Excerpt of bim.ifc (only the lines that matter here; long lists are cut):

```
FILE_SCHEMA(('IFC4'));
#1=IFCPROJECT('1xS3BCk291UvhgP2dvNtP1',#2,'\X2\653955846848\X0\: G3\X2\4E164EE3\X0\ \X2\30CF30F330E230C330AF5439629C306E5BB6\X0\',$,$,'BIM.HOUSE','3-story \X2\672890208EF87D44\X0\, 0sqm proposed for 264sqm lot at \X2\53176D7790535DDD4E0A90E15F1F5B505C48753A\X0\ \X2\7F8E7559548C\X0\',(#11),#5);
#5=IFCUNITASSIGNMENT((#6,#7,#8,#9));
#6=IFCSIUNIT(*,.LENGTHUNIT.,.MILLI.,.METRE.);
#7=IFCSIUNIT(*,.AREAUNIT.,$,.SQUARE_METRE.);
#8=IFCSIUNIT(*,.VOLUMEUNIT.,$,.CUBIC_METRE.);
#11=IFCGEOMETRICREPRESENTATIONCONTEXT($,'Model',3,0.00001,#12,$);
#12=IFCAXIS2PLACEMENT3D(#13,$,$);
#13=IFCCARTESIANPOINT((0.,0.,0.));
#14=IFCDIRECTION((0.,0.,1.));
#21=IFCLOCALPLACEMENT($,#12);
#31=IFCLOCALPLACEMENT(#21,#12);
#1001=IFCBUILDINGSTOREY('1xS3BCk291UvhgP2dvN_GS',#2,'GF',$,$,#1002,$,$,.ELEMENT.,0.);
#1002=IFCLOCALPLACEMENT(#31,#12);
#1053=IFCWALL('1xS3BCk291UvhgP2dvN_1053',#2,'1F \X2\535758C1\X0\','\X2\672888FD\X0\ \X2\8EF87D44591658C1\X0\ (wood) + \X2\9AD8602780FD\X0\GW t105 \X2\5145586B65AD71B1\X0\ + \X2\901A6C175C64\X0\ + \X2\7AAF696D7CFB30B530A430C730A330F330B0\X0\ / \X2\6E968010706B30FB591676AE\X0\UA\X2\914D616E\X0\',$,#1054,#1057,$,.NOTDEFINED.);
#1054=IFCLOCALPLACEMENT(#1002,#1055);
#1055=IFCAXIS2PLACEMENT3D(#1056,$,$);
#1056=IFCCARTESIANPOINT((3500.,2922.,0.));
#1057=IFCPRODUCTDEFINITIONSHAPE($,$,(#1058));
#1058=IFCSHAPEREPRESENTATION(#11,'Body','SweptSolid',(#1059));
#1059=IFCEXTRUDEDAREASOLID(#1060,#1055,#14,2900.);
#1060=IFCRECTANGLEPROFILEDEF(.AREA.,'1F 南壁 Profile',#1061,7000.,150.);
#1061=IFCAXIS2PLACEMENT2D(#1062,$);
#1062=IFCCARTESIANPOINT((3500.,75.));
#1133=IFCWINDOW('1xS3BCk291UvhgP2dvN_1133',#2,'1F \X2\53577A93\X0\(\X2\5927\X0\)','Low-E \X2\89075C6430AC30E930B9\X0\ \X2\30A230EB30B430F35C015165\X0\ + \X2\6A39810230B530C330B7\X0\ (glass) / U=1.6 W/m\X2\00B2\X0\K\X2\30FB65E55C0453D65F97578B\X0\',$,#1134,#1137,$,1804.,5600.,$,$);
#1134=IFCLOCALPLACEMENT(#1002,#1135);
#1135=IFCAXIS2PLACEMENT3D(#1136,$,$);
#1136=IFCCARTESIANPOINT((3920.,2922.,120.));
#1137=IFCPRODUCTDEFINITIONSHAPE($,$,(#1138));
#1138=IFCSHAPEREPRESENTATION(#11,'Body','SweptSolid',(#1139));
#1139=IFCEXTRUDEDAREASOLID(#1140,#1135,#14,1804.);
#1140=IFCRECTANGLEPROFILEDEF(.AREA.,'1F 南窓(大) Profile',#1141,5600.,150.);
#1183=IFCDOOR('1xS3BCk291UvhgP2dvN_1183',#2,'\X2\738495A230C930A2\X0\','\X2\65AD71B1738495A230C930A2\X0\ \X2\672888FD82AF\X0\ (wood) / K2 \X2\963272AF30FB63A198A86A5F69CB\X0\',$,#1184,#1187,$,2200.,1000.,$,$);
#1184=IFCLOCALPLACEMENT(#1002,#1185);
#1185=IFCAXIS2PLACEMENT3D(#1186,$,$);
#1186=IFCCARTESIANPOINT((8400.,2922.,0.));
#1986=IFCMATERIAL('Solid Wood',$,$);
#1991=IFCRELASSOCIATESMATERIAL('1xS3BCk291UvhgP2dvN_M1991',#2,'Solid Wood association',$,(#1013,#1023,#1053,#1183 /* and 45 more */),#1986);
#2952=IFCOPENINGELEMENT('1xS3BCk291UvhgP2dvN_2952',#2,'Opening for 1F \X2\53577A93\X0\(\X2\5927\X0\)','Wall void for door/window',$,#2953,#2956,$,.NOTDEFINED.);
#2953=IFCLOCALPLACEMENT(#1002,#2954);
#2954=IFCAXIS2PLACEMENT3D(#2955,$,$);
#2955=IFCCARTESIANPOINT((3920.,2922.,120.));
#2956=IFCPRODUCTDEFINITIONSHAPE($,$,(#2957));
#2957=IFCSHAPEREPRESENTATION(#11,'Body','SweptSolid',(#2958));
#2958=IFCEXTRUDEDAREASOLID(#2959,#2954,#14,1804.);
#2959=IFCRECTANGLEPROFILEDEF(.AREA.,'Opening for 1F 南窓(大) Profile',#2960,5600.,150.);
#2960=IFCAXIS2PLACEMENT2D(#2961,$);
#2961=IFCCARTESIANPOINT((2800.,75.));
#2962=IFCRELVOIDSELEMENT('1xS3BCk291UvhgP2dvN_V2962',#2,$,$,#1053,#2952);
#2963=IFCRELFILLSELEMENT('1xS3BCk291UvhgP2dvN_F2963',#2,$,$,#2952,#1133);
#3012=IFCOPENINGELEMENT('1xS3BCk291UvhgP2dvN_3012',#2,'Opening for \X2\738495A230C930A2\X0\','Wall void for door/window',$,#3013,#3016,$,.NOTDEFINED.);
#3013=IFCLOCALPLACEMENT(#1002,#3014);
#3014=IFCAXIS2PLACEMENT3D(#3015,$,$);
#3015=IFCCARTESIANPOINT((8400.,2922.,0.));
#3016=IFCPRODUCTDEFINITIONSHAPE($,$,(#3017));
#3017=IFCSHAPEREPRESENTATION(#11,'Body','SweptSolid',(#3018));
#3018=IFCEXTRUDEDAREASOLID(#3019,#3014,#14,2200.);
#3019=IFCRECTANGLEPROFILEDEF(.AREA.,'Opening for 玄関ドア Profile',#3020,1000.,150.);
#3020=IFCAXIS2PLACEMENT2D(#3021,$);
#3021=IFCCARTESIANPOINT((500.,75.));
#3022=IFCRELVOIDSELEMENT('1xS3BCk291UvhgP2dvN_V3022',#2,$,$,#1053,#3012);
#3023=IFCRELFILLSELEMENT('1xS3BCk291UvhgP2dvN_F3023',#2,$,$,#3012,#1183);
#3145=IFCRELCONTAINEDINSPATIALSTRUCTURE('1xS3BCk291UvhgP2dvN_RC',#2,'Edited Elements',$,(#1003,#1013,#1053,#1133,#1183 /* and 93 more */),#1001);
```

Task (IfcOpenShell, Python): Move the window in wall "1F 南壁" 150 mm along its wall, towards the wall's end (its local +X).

```python
import ifcopenshell
import ifcopenshell.api.geometry
import ifcopenshell.util.placement
import ifcopenshell.util.unit

model = ifcopenshell.open("bim.ifc")
unit_scale = ifcopenshell.util.unit.calculate_unit_scale(model)

window = model.by_guid("1xS3BCk291UvhgP2dvN_1133")
opening = window.FillsVoids[0].RelatingOpeningElement
wall = opening.VoidsElements[0].RelatingBuildingElement

wall_matrix = ifcopenshell.util.placement.get_local_placement(wall.ObjectPlacement)
shift = wall_matrix[:3, 0] * 0.15 / unit_scale
before = ifcopenshell.util.placement.get_local_placement(window.ObjectPlacement)[:3, 3].copy()

# The window is not placed relative to its opening, so move both.
for product in (opening, window):
    matrix = ifcopenshell.util.placement.get_local_placement(product.ObjectPlacement)
    matrix[:3, 3] += shift
    ifcopenshell.api.geometry.edit_object_placement(model, product=product, matrix=matrix, is_si=False)

after = ifcopenshell.util.placement.get_local_placement(window.ObjectPlacement)[:3, 3]
print("window moved by", (after - before).round(3) + 0.0)

model.write("bim_updated.ifc")
```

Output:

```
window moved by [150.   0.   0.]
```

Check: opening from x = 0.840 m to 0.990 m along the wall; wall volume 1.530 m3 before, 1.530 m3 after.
